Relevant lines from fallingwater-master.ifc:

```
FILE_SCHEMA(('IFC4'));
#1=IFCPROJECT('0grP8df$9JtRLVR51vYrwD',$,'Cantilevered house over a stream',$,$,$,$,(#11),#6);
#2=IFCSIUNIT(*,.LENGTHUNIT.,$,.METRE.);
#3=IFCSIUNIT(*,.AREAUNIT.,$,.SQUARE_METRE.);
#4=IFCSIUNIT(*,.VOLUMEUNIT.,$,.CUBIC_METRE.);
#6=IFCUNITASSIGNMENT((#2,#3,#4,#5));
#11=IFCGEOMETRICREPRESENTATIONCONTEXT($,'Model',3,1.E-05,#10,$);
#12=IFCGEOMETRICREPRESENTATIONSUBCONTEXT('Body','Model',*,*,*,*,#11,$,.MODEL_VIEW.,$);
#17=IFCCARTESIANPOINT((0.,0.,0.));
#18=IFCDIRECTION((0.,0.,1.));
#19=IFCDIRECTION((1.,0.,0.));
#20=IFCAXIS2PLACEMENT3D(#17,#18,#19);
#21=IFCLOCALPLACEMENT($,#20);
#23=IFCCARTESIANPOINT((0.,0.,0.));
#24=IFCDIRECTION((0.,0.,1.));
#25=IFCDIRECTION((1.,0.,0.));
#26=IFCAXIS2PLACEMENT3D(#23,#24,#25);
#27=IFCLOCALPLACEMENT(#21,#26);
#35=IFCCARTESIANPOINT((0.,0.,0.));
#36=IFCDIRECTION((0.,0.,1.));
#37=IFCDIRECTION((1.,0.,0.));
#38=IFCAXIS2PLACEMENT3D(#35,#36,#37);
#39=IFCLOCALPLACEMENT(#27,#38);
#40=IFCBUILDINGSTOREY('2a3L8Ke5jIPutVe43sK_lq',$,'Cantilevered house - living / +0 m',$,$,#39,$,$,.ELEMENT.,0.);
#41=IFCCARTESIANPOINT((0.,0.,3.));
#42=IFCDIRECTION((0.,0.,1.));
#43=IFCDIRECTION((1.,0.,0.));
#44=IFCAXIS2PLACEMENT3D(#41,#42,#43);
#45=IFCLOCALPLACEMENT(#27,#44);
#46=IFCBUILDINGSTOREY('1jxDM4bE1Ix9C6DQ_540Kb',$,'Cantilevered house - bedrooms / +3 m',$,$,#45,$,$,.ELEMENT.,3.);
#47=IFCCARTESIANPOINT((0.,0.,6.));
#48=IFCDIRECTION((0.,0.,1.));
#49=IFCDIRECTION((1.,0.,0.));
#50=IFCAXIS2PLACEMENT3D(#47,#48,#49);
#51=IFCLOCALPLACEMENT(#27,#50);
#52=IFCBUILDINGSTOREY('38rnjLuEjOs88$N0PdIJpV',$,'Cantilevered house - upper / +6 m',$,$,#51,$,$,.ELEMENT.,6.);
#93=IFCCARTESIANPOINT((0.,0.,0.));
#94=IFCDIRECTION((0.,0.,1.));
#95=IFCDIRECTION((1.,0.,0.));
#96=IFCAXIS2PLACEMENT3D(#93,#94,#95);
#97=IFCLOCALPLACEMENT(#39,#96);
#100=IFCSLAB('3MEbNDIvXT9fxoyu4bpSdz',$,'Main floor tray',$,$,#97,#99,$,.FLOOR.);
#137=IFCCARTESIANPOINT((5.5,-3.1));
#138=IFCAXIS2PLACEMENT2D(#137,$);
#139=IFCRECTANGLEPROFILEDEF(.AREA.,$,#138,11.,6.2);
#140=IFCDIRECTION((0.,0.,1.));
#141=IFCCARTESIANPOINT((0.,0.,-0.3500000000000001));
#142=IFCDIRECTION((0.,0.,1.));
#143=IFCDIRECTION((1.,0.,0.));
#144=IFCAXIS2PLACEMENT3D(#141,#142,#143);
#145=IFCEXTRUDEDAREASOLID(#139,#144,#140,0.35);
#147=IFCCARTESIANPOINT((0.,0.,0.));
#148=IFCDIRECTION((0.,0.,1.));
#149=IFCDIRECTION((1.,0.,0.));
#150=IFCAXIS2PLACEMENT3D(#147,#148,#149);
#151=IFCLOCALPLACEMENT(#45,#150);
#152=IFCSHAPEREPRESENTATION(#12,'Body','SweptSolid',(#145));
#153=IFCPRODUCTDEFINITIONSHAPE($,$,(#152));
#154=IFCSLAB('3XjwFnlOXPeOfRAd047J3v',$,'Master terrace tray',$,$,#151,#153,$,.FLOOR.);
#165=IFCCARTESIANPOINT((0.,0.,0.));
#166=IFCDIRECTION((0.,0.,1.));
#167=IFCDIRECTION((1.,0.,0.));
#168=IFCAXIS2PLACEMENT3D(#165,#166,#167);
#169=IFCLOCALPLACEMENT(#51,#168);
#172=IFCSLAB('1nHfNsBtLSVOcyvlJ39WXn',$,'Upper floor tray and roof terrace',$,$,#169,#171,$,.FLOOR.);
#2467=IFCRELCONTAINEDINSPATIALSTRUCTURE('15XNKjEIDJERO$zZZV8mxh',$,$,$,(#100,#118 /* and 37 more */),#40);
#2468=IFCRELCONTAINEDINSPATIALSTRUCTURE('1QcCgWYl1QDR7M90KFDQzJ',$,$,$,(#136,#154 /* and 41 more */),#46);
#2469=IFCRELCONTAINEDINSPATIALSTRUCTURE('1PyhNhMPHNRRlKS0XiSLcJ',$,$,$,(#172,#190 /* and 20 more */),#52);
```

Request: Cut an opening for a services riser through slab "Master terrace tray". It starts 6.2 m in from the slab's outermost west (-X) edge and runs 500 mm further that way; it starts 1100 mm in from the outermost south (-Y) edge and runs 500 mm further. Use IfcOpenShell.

```python
import numpy as np
import ifcopenshell
import ifcopenshell.api.feature
import ifcopenshell.api.geometry
import ifcopenshell.api.root
import ifcopenshell.geom
import ifcopenshell.util.placement
import ifcopenshell.util.representation
import ifcopenshell.util.shape
import ifcopenshell.util.unit

model = ifcopenshell.open("fallingwater-master.ifc")
unit_scale = ifcopenshell.util.unit.calculate_unit_scale(model)
settings = ifcopenshell.geom.settings()


def volume(element):
    """Net volume in cubic metres, openings subtracted."""
    shape = ifcopenshell.geom.create_shape(settings, element)
    return ifcopenshell.util.shape.get_volume(shape.geometry)


slab = model.by_id(154)
before = volume(slab)

# Extent in the slab's own axes, in metres. The edges named are its -X and -Y sides.
slab_shape = ifcopenshell.geom.create_shape(settings, slab)
vertices = ifcopenshell.util.shape.get_vertices(slab_shape.geometry)
x_min, y_min, bottom = vertices.min(axis=0)
top = vertices[:, 2].max()

opening = ifcopenshell.api.root.create_entity(model, ifc_class="IfcOpeningElement", name="Services riser opening", predefined_type="OPENING")
context = ifcopenshell.util.representation.get_context(model, "Model", "Body", "MODEL_VIEW")
width, depth = 0.5, 0.5
outline = [(0.0, 0.0), (width, 0.0), (width, depth), (0.0, depth), (0.0, 0.0)]
# Overshoot both faces by 50 mm so the cut is clean.
shape = ifcopenshell.api.geometry.add_slab_representation(
    model, context=context, depth=top - bottom + 0.1, polyline=outline
)
ifcopenshell.api.geometry.assign_representation(model, product=opening, representation=shape)

matrix = ifcopenshell.util.placement.get_local_placement(slab.ObjectPlacement)
matrix[:, 3] = matrix @ np.append(np.array([x_min + 6.2, y_min + 1.1, bottom - 0.05]) / unit_scale, 1.0)
ifcopenshell.api.geometry.edit_object_placement(model, product=opening, matrix=matrix, is_si=False)
ifcopenshell.api.feature.add_feature(model, feature=opening, element=slab)

after = volume(slab)

print(f"slab volume {before:.3f} -> {after:.3f} m3")

model.write("fallingwater-master_updated.ifc")
```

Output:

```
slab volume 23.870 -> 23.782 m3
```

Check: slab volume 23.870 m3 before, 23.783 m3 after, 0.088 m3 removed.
